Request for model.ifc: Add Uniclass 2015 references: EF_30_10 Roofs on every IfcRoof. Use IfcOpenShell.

First a look at what the model holds.

```python
import ifcopenshell

model = ifcopenshell.open("model.ifc")
print(model.schema)
print("classifications:", [c.Name for c in model.by_type("IfcClassification")])
for ifc_class in ("IfcDoor", "IfcRoof", "IfcStair", "IfcWall", "IfcWindow"):
    print(ifc_class, len(model.by_type(ifc_class)))
```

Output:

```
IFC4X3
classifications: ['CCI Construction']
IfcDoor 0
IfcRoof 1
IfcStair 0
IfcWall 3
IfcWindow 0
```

```python
import ifcopenshell
import ifcopenshell.api.classification

model = ifcopenshell.open("model.ifc")

system = ifcopenshell.api.classification.add_classification(model, classification="Uniclass 2015")

codes = {
    "IfcRoof": ("EF_30_10", "Roofs"),
}
for ifc_class, (code, name) in codes.items():
    products = model.by_type(ifc_class)
    ifcopenshell.api.classification.add_reference(
        model, products=products, classification=system, identification=code, name=name
    )
    print(code, len(products))

model.write("model_edited.ifc")
```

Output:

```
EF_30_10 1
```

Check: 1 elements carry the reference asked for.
